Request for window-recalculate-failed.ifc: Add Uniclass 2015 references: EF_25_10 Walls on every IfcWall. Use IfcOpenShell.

First a look at what the model holds.

```python
import ifcopenshell

model = ifcopenshell.open("window-recalculate-failed.ifc")
print(model.schema)
print("classifications:", [c.Name for c in model.by_type("IfcClassification")])
for ifc_class in ("IfcDoor", "IfcRoof", "IfcStair", "IfcWall", "IfcWindow"):
    print(ifc_class, len(model.by_type(ifc_class)))
```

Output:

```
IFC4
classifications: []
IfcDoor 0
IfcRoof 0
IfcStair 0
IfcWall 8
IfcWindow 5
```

```python
import ifcopenshell
import ifcopenshell.api.classification

model = ifcopenshell.open("window-recalculate-failed.ifc")

system = ifcopenshell.api.classification.add_classification(model, classification="Uniclass 2015")

codes = {
    "IfcWall": ("EF_25_10", "Walls"),
}
for ifc_class, (code, name) in codes.items():
    products = model.by_type(ifc_class)
    ifcopenshell.api.classification.add_reference(
        model, products=products, classification=system, identification=code, name=name
    )
    print(code, len(products))

model.write("window-recalculate-failed_v2.ifc")
```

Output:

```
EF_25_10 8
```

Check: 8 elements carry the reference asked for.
